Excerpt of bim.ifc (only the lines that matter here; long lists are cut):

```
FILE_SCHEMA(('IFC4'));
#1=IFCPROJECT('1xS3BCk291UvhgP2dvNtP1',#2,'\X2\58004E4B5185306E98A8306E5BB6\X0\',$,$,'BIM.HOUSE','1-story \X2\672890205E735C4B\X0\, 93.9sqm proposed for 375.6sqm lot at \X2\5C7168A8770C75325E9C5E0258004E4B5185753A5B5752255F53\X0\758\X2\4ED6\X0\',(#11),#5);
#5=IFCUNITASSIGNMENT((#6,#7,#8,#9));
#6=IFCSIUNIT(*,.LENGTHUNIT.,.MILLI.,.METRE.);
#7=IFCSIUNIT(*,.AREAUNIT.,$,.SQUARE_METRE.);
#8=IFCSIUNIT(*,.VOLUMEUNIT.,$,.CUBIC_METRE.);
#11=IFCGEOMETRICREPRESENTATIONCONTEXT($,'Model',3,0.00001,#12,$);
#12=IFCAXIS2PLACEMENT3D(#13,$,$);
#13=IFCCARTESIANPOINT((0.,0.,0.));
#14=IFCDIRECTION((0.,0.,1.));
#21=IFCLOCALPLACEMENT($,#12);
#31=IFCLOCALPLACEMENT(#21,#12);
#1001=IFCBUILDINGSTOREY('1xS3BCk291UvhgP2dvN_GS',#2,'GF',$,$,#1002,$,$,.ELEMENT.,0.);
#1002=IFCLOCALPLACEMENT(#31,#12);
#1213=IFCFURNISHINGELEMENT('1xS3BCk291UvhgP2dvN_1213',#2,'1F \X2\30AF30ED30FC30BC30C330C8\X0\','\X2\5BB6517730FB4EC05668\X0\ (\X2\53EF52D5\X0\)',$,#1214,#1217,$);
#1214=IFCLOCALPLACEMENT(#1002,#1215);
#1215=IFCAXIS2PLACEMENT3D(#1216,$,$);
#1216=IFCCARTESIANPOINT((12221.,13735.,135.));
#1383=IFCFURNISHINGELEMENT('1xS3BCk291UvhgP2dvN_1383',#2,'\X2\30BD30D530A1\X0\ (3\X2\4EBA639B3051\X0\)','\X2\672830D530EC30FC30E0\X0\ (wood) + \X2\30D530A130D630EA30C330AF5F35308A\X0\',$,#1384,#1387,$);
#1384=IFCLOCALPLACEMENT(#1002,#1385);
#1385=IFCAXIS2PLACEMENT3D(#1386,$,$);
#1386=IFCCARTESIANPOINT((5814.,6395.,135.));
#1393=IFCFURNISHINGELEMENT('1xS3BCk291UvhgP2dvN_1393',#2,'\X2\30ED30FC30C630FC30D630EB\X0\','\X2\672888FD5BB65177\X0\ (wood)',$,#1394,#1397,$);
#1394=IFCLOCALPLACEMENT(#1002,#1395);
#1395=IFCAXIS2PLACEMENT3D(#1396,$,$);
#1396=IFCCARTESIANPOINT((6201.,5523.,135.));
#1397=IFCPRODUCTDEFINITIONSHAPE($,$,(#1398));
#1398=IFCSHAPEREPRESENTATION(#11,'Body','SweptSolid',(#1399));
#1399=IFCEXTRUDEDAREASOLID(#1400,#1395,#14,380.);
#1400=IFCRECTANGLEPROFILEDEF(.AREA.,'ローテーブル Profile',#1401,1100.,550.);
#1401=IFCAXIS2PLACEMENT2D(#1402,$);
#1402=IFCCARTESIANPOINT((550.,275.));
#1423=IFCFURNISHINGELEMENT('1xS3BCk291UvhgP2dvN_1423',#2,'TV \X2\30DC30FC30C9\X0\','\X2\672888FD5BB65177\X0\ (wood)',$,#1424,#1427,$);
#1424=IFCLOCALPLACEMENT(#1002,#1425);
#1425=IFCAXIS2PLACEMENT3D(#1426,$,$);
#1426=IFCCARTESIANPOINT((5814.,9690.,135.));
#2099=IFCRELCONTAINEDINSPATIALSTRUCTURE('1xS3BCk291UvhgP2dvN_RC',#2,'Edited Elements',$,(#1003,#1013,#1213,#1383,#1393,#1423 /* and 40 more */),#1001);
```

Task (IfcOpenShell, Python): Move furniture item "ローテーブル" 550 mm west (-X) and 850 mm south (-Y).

```python
import ifcopenshell
import ifcopenshell.api.geometry
import ifcopenshell.util.placement

model = ifcopenshell.open("bim.ifc")

item = model.by_guid("1xS3BCk291UvhgP2dvN_1393")
matrix = ifcopenshell.util.placement.get_local_placement(item.ObjectPlacement)
matrix[0, 3] -= 550.0
matrix[1, 3] -= 850.0
ifcopenshell.api.geometry.edit_object_placement(model, product=item, matrix=matrix, is_si=False)

print(ifcopenshell.util.placement.get_local_placement(item.ObjectPlacement).round(3) + 0.0)

model.write("bim-out.ifc")
```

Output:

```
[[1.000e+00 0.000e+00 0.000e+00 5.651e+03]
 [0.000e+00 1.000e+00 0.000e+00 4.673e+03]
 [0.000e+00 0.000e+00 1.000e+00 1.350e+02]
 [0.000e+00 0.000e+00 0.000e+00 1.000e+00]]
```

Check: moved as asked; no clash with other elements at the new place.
